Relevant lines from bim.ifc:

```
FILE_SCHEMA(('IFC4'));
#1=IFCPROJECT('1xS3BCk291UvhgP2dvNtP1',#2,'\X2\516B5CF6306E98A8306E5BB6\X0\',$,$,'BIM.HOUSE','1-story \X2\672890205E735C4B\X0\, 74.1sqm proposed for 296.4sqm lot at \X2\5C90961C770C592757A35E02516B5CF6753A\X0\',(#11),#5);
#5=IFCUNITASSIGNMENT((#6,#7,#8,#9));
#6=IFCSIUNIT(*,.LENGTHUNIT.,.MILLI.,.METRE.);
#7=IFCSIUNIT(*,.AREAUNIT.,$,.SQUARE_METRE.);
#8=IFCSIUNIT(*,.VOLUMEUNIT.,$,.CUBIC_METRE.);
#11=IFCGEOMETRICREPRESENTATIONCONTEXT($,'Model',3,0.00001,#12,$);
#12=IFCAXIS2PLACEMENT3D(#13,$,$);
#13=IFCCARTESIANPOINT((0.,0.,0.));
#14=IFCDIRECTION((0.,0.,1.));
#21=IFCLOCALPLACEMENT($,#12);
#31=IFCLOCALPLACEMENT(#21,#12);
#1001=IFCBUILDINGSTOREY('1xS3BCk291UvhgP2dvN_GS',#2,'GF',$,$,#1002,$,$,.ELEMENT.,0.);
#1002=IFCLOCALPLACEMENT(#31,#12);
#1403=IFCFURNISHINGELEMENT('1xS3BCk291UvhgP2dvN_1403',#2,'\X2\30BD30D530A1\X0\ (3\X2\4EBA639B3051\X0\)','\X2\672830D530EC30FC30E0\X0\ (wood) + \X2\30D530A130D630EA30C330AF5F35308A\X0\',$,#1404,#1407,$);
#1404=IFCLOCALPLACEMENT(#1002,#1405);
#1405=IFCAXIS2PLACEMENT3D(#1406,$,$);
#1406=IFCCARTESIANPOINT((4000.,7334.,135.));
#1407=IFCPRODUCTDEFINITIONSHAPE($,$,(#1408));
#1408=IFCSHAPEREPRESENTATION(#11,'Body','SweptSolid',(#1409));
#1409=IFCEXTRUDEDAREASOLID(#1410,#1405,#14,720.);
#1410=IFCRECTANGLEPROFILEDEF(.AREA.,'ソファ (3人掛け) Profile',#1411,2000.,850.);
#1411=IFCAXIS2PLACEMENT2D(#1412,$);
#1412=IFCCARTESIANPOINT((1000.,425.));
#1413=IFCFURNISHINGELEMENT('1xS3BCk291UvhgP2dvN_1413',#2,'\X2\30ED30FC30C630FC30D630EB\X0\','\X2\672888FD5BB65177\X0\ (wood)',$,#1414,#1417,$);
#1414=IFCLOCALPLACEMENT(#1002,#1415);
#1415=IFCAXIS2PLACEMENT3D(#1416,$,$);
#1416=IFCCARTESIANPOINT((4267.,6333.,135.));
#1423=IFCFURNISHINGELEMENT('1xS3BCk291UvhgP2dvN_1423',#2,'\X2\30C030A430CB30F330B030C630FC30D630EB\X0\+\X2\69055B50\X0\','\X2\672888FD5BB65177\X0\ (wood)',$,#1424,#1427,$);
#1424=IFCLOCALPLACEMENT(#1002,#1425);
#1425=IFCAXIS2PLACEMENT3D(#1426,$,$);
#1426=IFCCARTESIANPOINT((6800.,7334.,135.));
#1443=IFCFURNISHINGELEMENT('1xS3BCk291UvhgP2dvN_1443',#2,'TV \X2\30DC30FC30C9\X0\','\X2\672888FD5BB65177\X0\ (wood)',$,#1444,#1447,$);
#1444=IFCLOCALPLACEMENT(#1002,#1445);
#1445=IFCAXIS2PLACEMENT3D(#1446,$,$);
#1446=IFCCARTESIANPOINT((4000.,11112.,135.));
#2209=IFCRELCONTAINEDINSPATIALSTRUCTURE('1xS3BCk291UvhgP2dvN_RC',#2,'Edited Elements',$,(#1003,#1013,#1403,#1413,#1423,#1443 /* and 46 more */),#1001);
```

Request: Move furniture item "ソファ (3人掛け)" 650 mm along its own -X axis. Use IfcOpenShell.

```python
import ifcopenshell
import ifcopenshell.api.geometry
import ifcopenshell.util.placement
import ifcopenshell.util.unit

model = ifcopenshell.open("bim.ifc")
unit_scale = ifcopenshell.util.unit.calculate_unit_scale(model)

item = model.by_guid("1xS3BCk291UvhgP2dvN_1403")
matrix = ifcopenshell.util.placement.get_local_placement(item.ObjectPlacement)
matrix[:3, 3] -= matrix[:3, 0] * 0.65 / unit_scale
ifcopenshell.api.geometry.edit_object_placement(model, product=item, matrix=matrix, is_si=False)

print(ifcopenshell.util.placement.get_local_placement(item.ObjectPlacement).round(3) + 0.0)

model.write("bim_updated.ifc")
```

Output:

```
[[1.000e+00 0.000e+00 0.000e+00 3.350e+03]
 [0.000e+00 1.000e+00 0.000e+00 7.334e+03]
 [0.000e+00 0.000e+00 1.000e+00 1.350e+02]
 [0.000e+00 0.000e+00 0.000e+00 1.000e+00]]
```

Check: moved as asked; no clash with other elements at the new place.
